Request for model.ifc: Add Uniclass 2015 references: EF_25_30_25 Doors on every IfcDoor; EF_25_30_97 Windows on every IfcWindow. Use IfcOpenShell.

First a look at what the model holds.

```python
import ifcopenshell

model = ifcopenshell.open("model.ifc")
print(model.schema)
print("classifications:", [c.Name for c in model.by_type("IfcClassification")])
for ifc_class in ("IfcDoor", "IfcRoof", "IfcStair", "IfcWall", "IfcWindow"):
    print(ifc_class, len(model.by_type(ifc_class)))
```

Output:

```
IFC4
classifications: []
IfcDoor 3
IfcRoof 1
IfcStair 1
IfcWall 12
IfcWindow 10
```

```python
import ifcopenshell
import ifcopenshell.api.classification

model = ifcopenshell.open("model.ifc")

system = ifcopenshell.api.classification.add_classification(model, classification="Uniclass 2015")

codes = {
    "IfcDoor": ("EF_25_30_25", "Doors"),
    "IfcWindow": ("EF_25_30_97", "Windows"),
}
for ifc_class, (code, name) in codes.items():
    products = model.by_type(ifc_class)
    ifcopenshell.api.classification.add_reference(
        model, products=products, classification=system, identification=code, name=name
    )
    print(code, len(products))

model.write("model_updated.ifc")
```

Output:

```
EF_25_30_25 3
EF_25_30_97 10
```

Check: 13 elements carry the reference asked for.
